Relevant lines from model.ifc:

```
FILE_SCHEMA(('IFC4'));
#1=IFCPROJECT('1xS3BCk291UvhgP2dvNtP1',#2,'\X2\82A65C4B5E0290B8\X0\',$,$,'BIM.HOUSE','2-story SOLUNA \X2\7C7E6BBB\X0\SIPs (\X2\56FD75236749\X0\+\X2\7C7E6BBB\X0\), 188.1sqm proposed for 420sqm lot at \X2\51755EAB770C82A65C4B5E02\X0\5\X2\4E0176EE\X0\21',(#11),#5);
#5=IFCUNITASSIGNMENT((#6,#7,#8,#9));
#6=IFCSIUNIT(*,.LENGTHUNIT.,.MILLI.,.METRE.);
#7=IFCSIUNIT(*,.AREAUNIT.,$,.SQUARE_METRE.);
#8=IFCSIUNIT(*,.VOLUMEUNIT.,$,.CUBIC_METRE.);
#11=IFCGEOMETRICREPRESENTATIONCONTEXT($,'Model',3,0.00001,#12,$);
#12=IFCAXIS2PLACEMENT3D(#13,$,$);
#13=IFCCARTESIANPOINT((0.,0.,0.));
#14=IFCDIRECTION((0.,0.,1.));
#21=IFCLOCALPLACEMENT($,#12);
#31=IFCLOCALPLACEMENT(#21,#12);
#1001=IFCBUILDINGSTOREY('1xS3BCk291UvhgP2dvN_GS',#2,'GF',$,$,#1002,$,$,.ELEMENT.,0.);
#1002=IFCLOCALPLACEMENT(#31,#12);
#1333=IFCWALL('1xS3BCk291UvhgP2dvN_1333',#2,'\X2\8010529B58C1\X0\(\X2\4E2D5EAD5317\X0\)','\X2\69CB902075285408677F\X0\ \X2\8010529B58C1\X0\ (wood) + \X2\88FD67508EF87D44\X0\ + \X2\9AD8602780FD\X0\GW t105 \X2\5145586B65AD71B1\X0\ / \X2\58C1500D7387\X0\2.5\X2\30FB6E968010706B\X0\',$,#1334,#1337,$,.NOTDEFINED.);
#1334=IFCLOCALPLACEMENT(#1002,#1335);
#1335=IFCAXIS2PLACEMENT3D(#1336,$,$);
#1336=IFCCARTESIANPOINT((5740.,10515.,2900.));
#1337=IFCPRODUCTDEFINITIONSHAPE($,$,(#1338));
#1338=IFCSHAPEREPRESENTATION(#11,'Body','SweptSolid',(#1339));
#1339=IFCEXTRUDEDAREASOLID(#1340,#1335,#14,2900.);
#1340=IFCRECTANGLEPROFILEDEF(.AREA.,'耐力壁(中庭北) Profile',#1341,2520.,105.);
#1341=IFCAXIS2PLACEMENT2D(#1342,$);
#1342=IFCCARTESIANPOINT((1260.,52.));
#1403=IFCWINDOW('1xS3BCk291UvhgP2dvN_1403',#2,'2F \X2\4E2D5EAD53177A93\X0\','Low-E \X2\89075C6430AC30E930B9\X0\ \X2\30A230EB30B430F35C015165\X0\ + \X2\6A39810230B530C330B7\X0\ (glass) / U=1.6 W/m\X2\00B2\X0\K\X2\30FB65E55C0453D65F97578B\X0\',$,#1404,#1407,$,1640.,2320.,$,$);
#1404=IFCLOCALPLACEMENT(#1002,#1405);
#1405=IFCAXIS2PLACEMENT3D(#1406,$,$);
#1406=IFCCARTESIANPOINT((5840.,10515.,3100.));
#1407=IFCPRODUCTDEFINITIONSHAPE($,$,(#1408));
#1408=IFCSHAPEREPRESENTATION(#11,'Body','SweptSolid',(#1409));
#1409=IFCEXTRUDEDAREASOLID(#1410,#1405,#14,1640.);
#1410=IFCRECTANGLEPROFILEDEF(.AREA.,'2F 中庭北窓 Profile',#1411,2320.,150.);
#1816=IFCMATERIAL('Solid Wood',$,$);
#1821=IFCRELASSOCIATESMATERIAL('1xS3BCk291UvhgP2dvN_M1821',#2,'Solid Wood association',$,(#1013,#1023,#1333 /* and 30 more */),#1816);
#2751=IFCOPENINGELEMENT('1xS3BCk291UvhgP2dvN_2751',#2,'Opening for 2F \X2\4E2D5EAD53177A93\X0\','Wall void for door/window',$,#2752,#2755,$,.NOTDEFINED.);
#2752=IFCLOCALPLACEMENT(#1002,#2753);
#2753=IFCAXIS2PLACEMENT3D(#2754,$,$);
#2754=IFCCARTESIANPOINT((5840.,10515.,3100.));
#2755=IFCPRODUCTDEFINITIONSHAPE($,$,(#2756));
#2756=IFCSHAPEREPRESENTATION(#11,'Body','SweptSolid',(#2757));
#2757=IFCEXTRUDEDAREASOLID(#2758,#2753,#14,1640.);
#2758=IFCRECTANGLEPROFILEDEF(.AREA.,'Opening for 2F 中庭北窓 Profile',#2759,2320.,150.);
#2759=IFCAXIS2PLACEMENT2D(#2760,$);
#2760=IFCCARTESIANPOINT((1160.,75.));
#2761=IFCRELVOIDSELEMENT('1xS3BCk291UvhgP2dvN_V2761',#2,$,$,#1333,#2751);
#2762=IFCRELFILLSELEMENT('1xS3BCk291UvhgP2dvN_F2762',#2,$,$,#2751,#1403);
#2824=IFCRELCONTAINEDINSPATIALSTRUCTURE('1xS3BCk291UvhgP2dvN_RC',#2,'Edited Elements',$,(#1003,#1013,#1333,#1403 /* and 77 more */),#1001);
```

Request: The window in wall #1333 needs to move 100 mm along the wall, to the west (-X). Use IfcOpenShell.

```python
import ifcopenshell
import ifcopenshell.api.geometry
import ifcopenshell.util.placement

model = ifcopenshell.open("model.ifc")

window = model.by_guid("1xS3BCk291UvhgP2dvN_1403")
opening = window.FillsVoids[0].RelatingOpeningElement
wall = opening.VoidsElements[0].RelatingBuildingElement

wall_matrix = ifcopenshell.util.placement.get_local_placement(wall.ObjectPlacement)
shift = wall_matrix[:3, 0] * -100.0
before = ifcopenshell.util.placement.get_local_placement(window.ObjectPlacement)[:3, 3].copy()

# The window is not placed relative to its opening, so move both.
for product in (opening, window):
    matrix = ifcopenshell.util.placement.get_local_placement(product.ObjectPlacement)
    matrix[:3, 3] += shift
    ifcopenshell.api.geometry.edit_object_placement(model, product=product, matrix=matrix, is_si=False)

after = ifcopenshell.util.placement.get_local_placement(window.ObjectPlacement)[:3, 3]
print("window moved by", (after - before).round(3) + 0.0)

model.write("model_rev.ifc")
```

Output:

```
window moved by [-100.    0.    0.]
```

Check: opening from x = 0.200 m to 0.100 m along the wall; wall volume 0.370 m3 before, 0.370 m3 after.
